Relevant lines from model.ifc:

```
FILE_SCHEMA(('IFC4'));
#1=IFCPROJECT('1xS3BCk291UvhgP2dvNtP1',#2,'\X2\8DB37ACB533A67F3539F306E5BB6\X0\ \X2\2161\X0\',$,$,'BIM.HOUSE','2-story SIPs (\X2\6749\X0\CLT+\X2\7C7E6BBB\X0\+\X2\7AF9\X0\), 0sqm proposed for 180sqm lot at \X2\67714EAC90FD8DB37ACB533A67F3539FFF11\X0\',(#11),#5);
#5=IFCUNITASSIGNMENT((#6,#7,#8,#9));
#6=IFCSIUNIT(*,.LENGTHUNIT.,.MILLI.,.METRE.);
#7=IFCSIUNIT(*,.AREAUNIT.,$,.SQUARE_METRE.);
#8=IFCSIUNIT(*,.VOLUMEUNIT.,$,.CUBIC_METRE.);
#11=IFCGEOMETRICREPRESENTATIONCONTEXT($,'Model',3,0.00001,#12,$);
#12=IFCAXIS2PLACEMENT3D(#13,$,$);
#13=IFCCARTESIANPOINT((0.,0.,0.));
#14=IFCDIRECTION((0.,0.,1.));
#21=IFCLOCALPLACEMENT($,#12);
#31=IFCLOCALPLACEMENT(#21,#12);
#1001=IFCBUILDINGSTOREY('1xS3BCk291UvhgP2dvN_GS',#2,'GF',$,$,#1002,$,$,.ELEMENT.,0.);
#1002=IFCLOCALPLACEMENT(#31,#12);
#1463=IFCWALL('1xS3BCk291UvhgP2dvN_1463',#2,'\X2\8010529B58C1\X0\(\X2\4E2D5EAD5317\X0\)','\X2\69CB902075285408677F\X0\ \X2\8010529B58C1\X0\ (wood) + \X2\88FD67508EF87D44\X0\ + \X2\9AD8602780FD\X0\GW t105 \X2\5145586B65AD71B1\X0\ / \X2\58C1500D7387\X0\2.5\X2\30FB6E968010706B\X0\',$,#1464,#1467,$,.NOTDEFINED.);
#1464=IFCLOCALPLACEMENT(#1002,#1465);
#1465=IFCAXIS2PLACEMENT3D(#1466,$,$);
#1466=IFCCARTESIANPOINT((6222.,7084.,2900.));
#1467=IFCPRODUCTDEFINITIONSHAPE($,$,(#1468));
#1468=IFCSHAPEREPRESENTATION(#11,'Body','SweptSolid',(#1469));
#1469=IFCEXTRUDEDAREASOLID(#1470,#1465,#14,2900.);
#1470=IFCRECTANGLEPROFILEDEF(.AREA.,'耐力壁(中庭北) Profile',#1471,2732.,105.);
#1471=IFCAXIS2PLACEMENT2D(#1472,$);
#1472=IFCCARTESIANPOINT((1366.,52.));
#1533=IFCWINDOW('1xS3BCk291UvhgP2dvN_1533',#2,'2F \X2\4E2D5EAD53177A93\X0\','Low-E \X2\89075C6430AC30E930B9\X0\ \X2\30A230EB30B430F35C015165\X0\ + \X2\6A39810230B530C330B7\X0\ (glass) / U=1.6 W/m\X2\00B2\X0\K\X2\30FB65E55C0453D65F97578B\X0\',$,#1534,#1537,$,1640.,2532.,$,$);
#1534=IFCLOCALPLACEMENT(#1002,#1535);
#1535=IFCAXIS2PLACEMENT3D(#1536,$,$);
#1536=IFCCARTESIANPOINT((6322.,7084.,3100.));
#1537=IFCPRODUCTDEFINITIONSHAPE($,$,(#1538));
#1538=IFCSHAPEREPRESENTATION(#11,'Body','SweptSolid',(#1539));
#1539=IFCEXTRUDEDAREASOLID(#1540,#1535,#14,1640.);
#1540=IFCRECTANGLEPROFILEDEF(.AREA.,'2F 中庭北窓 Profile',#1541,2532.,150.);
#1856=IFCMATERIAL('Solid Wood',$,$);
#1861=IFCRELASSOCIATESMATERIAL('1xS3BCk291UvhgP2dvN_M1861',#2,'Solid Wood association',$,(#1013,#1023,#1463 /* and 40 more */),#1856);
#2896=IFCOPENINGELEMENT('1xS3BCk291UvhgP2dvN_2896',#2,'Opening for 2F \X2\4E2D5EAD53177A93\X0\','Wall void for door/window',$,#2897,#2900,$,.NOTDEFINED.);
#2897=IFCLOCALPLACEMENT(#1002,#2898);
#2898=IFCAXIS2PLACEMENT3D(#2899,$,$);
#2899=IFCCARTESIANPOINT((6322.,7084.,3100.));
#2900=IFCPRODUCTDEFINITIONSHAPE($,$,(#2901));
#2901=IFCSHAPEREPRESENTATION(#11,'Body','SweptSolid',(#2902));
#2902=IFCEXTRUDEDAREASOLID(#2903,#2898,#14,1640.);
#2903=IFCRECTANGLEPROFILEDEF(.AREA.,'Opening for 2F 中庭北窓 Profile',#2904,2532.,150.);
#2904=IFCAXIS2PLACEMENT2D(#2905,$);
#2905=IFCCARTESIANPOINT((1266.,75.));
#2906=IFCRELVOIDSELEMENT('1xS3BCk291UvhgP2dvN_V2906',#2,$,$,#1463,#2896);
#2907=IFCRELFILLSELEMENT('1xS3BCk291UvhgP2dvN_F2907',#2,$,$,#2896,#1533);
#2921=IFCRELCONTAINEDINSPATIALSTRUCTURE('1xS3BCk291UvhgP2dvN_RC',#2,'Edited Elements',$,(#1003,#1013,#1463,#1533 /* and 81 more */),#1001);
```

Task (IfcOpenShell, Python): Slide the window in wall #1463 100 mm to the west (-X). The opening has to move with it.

```python
import ifcopenshell
import ifcopenshell.api.geometry
import ifcopenshell.util.placement

model = ifcopenshell.open("model.ifc")

window = model.by_id(1533)
opening = window.FillsVoids[0].RelatingOpeningElement
wall = opening.VoidsElements[0].RelatingBuildingElement

wall_matrix = ifcopenshell.util.placement.get_local_placement(wall.ObjectPlacement)
shift = wall_matrix[:3, 0] * -100.0
before = ifcopenshell.util.placement.get_local_placement(window.ObjectPlacement)[:3, 3].copy()

# The window is not placed relative to its opening, so move both.
for product in (opening, window):
    matrix = ifcopenshell.util.placement.get_local_placement(product.ObjectPlacement)
    matrix[:3, 3] += shift
    ifcopenshell.api.geometry.edit_object_placement(model, product=product, matrix=matrix, is_si=False)

after = ifcopenshell.util.placement.get_local_placement(window.ObjectPlacement)[:3, 3]
print("window moved by", (after - before).round(3) + 0.0)

model.write("model_rev.ifc")
```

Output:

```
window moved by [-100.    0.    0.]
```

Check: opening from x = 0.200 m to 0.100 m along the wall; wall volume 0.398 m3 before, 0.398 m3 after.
